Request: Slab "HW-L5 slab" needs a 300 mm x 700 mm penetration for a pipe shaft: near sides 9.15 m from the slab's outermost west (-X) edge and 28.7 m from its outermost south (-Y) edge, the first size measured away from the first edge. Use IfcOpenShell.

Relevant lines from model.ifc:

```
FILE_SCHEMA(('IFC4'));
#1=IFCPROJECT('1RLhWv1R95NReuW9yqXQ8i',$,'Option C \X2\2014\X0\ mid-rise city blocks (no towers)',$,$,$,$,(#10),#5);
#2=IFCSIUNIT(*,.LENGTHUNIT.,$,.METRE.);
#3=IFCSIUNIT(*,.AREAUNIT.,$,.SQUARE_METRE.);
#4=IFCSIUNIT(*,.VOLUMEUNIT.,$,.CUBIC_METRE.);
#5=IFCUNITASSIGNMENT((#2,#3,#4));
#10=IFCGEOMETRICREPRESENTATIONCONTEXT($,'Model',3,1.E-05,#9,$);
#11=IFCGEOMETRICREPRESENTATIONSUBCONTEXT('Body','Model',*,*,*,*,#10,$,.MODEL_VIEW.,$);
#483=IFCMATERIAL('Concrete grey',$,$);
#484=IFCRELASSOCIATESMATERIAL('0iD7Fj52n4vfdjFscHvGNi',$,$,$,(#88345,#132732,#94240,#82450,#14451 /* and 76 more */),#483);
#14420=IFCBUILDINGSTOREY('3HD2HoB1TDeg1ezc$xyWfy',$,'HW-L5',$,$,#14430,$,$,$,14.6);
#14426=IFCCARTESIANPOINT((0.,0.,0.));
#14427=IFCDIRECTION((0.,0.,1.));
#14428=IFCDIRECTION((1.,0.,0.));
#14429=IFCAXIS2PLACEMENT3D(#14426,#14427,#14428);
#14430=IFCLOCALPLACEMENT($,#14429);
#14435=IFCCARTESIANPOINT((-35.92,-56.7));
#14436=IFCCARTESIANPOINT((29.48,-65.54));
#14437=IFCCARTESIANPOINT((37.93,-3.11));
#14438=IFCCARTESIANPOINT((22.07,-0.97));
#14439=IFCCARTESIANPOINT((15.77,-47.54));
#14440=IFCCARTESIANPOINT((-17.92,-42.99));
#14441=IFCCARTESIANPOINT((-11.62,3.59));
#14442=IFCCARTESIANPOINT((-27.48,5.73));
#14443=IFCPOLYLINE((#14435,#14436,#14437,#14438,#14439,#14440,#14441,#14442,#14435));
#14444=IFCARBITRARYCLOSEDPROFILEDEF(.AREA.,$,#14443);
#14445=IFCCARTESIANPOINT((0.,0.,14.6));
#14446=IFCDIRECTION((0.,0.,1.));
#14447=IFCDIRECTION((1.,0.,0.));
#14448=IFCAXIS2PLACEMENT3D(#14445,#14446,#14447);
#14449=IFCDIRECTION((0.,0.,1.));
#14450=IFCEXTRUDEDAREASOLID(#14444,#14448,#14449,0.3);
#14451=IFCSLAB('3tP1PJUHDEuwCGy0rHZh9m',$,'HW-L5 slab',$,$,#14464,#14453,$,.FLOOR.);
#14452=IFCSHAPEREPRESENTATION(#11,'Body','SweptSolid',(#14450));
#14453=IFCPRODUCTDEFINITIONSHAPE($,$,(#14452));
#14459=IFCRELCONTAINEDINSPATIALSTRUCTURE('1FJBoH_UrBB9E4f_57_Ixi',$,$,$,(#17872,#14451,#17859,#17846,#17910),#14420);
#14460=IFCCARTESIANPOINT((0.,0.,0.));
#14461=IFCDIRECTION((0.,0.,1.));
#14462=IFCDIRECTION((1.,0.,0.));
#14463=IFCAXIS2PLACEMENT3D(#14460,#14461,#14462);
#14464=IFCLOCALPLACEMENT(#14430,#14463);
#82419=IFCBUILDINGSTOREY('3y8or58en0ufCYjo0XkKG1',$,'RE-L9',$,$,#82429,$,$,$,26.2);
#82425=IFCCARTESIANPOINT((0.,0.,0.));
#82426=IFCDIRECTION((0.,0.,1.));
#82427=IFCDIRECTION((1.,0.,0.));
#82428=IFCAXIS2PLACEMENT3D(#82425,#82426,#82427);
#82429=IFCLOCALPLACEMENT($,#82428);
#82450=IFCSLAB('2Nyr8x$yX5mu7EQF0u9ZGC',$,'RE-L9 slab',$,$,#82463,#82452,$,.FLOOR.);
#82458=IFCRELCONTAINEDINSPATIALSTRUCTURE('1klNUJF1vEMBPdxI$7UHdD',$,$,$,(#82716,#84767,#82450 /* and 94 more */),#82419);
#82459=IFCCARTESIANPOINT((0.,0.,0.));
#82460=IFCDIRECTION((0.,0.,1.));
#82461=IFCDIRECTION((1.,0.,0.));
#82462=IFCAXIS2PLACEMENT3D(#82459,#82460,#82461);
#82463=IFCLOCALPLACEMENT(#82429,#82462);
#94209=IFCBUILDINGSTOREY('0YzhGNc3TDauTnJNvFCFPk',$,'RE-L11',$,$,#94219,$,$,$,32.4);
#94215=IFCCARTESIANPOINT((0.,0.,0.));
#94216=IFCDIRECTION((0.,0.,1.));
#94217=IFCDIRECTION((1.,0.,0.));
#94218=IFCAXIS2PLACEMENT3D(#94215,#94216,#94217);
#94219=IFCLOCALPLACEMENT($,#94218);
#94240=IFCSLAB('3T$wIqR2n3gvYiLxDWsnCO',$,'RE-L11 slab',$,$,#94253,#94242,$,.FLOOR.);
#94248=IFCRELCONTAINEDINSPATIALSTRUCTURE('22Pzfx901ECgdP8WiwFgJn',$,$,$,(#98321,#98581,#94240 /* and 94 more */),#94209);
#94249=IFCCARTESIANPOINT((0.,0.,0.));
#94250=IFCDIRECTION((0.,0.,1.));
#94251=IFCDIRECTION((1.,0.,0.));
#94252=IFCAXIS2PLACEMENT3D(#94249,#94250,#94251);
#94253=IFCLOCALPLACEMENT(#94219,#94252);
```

```python
import numpy as np
import ifcopenshell
import ifcopenshell.api.feature
import ifcopenshell.api.geometry
import ifcopenshell.api.root
import ifcopenshell.geom
import ifcopenshell.util.placement
import ifcopenshell.util.representation
import ifcopenshell.util.shape
import ifcopenshell.util.unit

model = ifcopenshell.open("model.ifc")
unit_scale = ifcopenshell.util.unit.calculate_unit_scale(model)
settings = ifcopenshell.geom.settings()


def volume(element):
    """Net volume in cubic metres, openings subtracted."""
    shape = ifcopenshell.geom.create_shape(settings, element)
    return ifcopenshell.util.shape.get_volume(shape.geometry)


slab = model.by_guid("3tP1PJUHDEuwCGy0rHZh9m")
before = volume(slab)

# Extent in the slab's own axes, in metres. The edges named are its -X and -Y sides.
slab_shape = ifcopenshell.geom.create_shape(settings, slab)
vertices = ifcopenshell.util.shape.get_vertices(slab_shape.geometry)
x_min, y_min, bottom = vertices.min(axis=0)
top = vertices[:, 2].max()

opening = ifcopenshell.api.root.create_entity(model, ifc_class="IfcOpeningElement", name="Pipe shaft opening", predefined_type="OPENING")
context = ifcopenshell.util.representation.get_context(model, "Model", "Body", "MODEL_VIEW")
width, depth = 0.3, 0.7
outline = [(0.0, 0.0), (width, 0.0), (width, depth), (0.0, depth), (0.0, 0.0)]
# Overshoot both faces by 50 mm so the cut is clean.
shape = ifcopenshell.api.geometry.add_slab_representation(
    model, context=context, depth=top - bottom + 0.1, polyline=outline
)
ifcopenshell.api.geometry.assign_representation(model, product=opening, representation=shape)

matrix = ifcopenshell.util.placement.get_local_placement(slab.ObjectPlacement)
matrix[:, 3] = matrix @ np.append(np.array([x_min + 9.15, y_min + 28.7, bottom - 0.05]) / unit_scale, 1.0)
ifcopenshell.api.geometry.edit_object_placement(model, product=opening, matrix=matrix, is_si=False)
ifcopenshell.api.feature.add_feature(model, feature=opening, element=slab)

after = volume(slab)

print(f"slab volume {before:.3f} -> {after:.3f} m3")

model.write("model-out.ifc")
```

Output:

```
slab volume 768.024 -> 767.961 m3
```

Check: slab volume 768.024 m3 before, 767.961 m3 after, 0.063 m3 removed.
